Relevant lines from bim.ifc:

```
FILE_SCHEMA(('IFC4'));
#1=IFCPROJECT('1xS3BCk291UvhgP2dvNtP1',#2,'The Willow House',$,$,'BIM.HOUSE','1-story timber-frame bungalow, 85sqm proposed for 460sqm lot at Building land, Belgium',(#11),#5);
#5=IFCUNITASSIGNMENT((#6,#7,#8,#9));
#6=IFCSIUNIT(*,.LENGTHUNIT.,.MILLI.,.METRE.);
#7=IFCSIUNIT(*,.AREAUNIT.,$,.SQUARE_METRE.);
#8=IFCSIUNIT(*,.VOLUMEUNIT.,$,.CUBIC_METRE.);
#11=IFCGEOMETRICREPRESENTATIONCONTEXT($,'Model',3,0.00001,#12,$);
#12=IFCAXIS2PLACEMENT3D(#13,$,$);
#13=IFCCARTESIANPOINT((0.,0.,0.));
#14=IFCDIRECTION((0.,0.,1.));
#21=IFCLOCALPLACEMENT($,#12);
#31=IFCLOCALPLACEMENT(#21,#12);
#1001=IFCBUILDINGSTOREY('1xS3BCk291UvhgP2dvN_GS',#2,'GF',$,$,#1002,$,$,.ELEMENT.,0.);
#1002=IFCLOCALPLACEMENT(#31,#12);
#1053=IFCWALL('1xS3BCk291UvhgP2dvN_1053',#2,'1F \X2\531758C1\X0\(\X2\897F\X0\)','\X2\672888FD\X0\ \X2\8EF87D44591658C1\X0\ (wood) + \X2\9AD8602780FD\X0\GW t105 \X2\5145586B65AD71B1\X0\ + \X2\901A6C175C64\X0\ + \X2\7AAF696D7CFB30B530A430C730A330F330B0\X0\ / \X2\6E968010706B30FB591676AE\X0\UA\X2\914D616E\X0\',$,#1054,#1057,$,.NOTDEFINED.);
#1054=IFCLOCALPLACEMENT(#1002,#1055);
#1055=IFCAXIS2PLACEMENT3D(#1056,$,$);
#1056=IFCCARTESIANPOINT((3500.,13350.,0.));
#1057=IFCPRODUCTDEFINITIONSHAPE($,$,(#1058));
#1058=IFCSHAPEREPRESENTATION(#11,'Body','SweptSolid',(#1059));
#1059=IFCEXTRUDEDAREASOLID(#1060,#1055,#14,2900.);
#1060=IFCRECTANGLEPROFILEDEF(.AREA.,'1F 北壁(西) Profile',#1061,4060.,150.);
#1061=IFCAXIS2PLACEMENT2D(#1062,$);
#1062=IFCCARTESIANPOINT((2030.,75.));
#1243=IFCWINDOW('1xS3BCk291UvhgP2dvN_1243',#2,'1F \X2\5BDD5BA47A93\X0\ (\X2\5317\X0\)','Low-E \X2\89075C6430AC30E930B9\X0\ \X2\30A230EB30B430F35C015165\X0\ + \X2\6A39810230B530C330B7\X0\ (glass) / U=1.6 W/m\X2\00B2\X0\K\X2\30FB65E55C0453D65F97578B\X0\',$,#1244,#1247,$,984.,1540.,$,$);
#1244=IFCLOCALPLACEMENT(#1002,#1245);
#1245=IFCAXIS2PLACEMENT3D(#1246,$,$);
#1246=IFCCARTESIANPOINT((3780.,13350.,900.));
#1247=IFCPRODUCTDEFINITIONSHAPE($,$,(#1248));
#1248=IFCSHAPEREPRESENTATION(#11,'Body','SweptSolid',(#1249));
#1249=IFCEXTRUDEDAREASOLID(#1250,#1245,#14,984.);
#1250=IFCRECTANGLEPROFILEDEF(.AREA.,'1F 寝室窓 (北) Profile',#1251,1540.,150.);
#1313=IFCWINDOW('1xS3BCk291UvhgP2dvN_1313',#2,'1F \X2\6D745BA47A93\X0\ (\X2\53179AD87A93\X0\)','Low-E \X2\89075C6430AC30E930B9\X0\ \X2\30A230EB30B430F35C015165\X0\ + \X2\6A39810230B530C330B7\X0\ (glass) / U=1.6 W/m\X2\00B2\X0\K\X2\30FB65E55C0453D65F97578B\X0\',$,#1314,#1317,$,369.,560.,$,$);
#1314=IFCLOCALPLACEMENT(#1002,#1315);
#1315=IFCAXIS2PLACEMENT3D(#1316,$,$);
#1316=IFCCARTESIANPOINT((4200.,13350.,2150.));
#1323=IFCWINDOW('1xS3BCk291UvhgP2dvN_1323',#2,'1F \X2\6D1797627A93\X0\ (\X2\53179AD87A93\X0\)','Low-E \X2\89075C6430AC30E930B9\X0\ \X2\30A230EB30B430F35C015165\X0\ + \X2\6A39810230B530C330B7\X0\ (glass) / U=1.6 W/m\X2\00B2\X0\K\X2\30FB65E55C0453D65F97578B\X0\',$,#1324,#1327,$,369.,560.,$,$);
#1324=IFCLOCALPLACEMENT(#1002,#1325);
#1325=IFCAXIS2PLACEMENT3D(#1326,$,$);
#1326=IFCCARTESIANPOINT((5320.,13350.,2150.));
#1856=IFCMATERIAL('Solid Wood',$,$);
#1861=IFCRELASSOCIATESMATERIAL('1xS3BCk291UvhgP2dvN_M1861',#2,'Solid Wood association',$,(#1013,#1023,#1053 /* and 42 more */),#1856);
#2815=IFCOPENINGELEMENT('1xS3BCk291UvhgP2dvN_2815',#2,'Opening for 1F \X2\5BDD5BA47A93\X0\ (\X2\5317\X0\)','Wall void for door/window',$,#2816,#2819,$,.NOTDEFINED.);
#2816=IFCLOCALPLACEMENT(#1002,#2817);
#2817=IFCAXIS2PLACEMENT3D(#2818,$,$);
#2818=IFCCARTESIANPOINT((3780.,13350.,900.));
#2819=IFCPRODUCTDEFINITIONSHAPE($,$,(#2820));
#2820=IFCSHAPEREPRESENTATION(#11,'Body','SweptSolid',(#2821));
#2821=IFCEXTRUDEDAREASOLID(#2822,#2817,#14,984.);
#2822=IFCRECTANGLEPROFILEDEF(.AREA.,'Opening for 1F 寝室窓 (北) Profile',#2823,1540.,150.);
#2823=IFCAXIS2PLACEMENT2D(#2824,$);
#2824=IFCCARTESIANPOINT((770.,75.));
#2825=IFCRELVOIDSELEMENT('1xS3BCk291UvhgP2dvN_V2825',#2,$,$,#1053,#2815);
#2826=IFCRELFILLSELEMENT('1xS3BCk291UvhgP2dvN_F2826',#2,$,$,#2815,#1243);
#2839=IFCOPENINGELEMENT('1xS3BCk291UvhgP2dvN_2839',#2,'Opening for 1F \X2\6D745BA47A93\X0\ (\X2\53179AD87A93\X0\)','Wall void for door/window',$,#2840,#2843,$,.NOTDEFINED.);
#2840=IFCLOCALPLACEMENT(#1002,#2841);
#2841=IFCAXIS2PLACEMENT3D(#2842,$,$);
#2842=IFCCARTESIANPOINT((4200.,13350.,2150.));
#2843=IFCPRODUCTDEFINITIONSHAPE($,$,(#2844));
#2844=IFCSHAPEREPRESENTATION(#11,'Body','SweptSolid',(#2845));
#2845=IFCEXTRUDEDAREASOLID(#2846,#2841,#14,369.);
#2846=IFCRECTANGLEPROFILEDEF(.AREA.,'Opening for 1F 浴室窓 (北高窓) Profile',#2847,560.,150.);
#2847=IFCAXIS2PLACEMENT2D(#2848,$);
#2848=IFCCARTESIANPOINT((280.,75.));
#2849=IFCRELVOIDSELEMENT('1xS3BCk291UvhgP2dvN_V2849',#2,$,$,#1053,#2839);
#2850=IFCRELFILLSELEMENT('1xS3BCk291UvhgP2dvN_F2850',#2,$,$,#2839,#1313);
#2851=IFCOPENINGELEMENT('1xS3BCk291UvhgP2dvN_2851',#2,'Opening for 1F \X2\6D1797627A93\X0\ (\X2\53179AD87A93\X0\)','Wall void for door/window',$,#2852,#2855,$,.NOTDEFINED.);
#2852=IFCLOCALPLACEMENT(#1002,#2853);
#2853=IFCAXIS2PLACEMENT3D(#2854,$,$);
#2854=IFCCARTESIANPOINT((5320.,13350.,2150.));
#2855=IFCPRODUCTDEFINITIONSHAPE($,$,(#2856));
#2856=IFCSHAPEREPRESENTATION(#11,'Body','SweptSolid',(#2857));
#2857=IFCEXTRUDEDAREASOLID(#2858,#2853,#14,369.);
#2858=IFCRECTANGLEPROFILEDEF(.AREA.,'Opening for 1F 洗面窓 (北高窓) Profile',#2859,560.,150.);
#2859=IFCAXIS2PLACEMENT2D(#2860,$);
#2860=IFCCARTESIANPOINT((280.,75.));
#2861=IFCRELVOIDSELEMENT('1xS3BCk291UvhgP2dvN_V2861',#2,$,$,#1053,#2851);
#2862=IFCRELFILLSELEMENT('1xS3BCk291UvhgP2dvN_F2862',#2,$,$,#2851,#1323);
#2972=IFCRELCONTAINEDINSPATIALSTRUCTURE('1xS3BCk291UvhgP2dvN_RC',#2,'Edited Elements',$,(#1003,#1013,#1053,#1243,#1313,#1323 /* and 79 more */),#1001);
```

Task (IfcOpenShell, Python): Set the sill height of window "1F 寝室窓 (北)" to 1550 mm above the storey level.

```python
import numpy as np
import ifcopenshell
import ifcopenshell.api.geometry
import ifcopenshell.geom
import ifcopenshell.util.element
import ifcopenshell.util.placement
import ifcopenshell.util.shape
import ifcopenshell.util.unit

model = ifcopenshell.open("bim.ifc")
unit_scale = ifcopenshell.util.unit.calculate_unit_scale(model)

window = model.by_guid("1xS3BCk291UvhgP2dvN_1243")
opening = window.FillsVoids[0].RelatingOpeningElement
storey = ifcopenshell.util.element.get_container(window, ifc_class="IfcBuildingStorey")
level = ifcopenshell.util.placement.get_local_placement(storey.ObjectPlacement)[2, 3]

# The opening's origin need not be at the sill, so measure its lowest point.
shape = ifcopenshell.geom.create_shape(ifcopenshell.geom.settings(), opening)
bottom = ifcopenshell.util.shape.get_shape_bottom_elevation(shape, shape.geometry) / unit_scale
dz = level + 1.55 / unit_scale - bottom

shift = np.array([0.0, 0.0, dz])
# The window is not placed relative to its opening, so move both.
for product in (opening, window):
    matrix = ifcopenshell.util.placement.get_local_placement(product.ObjectPlacement)
    matrix[:3, 3] += shift
    ifcopenshell.api.geometry.edit_object_placement(model, product=product, matrix=matrix, is_si=False)

print(f"moved by {dz * unit_scale:+.3f} m")

model.write("bim-out.ifc")
```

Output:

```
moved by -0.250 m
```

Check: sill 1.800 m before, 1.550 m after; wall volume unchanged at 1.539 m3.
